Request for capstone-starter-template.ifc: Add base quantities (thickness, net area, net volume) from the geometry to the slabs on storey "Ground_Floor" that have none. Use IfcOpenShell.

First a look at what the model holds.

```python
import ifcopenshell
import ifcopenshell.util.element
import ifcopenshell.util.unit

model = ifcopenshell.open("capstone-starter-template.ifc")
print(model.schema)
for unit_type in ("LENGTHUNIT", "AREAUNIT", "VOLUMEUNIT"):
    print(unit_type, ifcopenshell.util.unit.calculate_unit_scale(model, unit_type))
storey = next(s for s in model.by_type("IfcBuildingStorey") if s.Name == "Ground_Floor")
slabs = [e for e in ifcopenshell.util.element.get_decomposition(storey) if e.is_a("IfcSlab")]
for e in sorted(slabs, key=lambda e: e.id()):
    print(e.id(), e.is_a(), e.Name, list(ifcopenshell.util.element.get_psets(e, qtos_only=True)), sep=" | ")
```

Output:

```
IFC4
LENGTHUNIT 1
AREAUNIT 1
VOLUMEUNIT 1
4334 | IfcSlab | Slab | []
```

```python
import ifcopenshell
import ifcopenshell.api.pset
import ifcopenshell.geom
import ifcopenshell.util.element
import ifcopenshell.util.shape
import ifcopenshell.util.unit

model = ifcopenshell.open("capstone-starter-template.ifc")
unit_scale = ifcopenshell.util.unit.calculate_unit_scale(model)
area_scale = ifcopenshell.util.unit.calculate_unit_scale(model, "AREAUNIT")
volume_scale = ifcopenshell.util.unit.calculate_unit_scale(model, "VOLUMEUNIT")
settings = ifcopenshell.geom.settings()

storey = next(s for s in model.by_type("IfcBuildingStorey") if s.Name == "Ground_Floor")
slabs = [e for e in ifcopenshell.util.element.get_decomposition(storey) if e.is_a("IfcSlab")]

for e in sorted(slabs, key=lambda e: e.id()):
    if ifcopenshell.util.element.get_psets(e, qtos_only=True, should_inherit=False):
        continue
    # Geometry comes back in metres, in the element's own axes.
    shape = ifcopenshell.geom.create_shape(settings, e)
    values = {
        "Width": ifcopenshell.util.shape.get_z(shape.geometry) / unit_scale,
        "NetArea": ifcopenshell.util.shape.get_footprint_area(shape.geometry) / area_scale,
        "NetVolume": ifcopenshell.util.shape.get_volume(shape.geometry) / volume_scale,
    }
    qto = ifcopenshell.api.pset.add_qto(model, product=e, name="Qto_SlabBaseQuantities")
    ifcopenshell.api.pset.edit_qto(model, qto=qto, properties=values)
    print(e.id(), {k: round(v, 3) for k, v in values.items()})

model.write("capstone-starter-template-out.ifc")
```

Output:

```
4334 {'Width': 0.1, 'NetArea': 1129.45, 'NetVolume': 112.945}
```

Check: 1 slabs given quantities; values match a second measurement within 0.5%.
